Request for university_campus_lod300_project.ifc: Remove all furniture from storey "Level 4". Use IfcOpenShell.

First a look at what the model holds.

```python
import ifcopenshell
import ifcopenshell.util.element

model = ifcopenshell.open("university_campus_lod300_project.ifc")
print(model.schema)
storey = next(s for s in model.by_type("IfcBuildingStorey") if s.Name == "Level 4")
furniture = [e for e in ifcopenshell.util.element.get_decomposition(storey) if e.is_a("IfcFurnishingElement")]
seen = {}
for e in furniture:
    element_type = ifcopenshell.util.element.get_type(e)
    name = element_type.Name if element_type not in (None, e) else None
    seen[name] = seen.get(name, 0) + 1
for name, count in sorted(seen.items(), key=str):
    print(count, "x", name)
```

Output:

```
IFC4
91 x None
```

```python
import ifcopenshell
import ifcopenshell.api.root
import ifcopenshell.util.element

model = ifcopenshell.open("university_campus_lod300_project.ifc")

storey = next(s for s in model.by_type("IfcBuildingStorey") if s.Name == "Level 4")
furniture = [e for e in ifcopenshell.util.element.get_decomposition(storey) if e.is_a("IfcFurnishingElement")]

for e in furniture:
    ifcopenshell.api.root.remove_product(model, product=e)
print(len(furniture), "removed")

model.write("university_campus_lod300_project_updated.ifc")
```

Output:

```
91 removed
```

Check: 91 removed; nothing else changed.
